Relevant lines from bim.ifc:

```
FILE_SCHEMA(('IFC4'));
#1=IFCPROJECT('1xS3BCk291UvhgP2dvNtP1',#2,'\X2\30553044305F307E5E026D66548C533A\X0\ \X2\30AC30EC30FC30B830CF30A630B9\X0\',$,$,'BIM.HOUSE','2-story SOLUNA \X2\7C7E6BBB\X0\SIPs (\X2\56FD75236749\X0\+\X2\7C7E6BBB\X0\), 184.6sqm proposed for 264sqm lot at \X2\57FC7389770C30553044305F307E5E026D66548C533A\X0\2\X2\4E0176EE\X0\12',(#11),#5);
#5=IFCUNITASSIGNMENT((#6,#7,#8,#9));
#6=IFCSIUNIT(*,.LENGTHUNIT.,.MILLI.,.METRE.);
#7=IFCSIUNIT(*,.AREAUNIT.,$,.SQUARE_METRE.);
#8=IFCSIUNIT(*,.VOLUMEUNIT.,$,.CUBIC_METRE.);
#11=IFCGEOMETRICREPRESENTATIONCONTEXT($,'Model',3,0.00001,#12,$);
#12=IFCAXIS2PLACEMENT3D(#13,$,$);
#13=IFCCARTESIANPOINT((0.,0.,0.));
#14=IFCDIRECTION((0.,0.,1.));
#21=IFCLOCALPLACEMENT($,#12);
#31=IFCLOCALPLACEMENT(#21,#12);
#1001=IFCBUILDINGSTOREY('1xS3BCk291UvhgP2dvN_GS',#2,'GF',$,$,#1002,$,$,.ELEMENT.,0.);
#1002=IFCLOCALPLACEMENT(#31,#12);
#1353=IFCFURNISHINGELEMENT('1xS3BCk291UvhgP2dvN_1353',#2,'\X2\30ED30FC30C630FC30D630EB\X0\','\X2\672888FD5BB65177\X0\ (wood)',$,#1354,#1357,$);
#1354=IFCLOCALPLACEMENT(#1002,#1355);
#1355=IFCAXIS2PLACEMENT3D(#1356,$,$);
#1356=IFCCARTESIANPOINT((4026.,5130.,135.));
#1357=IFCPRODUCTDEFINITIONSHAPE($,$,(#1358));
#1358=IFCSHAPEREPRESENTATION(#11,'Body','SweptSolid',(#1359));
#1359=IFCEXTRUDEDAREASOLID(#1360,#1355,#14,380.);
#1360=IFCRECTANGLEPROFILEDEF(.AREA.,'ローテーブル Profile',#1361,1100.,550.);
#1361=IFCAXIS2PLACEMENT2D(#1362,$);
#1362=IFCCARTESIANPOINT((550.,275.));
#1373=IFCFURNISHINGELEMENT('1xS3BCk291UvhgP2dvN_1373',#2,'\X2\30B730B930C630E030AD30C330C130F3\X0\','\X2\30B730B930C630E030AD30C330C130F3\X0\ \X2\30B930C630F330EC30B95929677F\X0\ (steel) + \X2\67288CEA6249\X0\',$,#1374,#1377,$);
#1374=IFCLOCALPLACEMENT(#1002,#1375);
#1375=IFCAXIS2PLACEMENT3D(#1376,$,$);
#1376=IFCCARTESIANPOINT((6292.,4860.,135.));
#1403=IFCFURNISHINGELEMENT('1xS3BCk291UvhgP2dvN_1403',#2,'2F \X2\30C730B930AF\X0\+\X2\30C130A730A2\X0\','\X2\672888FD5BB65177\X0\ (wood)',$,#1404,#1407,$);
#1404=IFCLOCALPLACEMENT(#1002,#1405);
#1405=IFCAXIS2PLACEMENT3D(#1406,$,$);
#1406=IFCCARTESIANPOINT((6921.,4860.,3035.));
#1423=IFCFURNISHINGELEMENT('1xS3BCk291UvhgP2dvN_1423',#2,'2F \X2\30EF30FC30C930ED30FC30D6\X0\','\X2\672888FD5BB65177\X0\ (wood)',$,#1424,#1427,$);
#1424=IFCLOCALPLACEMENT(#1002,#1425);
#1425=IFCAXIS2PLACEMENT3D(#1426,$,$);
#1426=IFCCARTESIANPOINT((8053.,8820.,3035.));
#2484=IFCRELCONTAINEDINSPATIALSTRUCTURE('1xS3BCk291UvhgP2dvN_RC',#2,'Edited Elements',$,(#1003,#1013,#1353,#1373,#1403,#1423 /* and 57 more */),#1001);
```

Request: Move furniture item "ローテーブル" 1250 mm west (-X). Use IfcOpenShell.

```python
import ifcopenshell
import ifcopenshell.api.geometry
import ifcopenshell.util.placement

model = ifcopenshell.open("bim.ifc")

item = model.by_id(1353)
matrix = ifcopenshell.util.placement.get_local_placement(item.ObjectPlacement)
matrix[0, 3] -= 1250.0
ifcopenshell.api.geometry.edit_object_placement(model, product=item, matrix=matrix, is_si=False)

print(ifcopenshell.util.placement.get_local_placement(item.ObjectPlacement).round(3) + 0.0)

model.write("bim_rev.ifc")
```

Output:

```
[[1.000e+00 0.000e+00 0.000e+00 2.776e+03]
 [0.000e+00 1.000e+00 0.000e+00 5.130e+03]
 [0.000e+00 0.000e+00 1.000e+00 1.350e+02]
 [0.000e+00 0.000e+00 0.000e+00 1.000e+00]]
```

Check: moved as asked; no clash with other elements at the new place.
